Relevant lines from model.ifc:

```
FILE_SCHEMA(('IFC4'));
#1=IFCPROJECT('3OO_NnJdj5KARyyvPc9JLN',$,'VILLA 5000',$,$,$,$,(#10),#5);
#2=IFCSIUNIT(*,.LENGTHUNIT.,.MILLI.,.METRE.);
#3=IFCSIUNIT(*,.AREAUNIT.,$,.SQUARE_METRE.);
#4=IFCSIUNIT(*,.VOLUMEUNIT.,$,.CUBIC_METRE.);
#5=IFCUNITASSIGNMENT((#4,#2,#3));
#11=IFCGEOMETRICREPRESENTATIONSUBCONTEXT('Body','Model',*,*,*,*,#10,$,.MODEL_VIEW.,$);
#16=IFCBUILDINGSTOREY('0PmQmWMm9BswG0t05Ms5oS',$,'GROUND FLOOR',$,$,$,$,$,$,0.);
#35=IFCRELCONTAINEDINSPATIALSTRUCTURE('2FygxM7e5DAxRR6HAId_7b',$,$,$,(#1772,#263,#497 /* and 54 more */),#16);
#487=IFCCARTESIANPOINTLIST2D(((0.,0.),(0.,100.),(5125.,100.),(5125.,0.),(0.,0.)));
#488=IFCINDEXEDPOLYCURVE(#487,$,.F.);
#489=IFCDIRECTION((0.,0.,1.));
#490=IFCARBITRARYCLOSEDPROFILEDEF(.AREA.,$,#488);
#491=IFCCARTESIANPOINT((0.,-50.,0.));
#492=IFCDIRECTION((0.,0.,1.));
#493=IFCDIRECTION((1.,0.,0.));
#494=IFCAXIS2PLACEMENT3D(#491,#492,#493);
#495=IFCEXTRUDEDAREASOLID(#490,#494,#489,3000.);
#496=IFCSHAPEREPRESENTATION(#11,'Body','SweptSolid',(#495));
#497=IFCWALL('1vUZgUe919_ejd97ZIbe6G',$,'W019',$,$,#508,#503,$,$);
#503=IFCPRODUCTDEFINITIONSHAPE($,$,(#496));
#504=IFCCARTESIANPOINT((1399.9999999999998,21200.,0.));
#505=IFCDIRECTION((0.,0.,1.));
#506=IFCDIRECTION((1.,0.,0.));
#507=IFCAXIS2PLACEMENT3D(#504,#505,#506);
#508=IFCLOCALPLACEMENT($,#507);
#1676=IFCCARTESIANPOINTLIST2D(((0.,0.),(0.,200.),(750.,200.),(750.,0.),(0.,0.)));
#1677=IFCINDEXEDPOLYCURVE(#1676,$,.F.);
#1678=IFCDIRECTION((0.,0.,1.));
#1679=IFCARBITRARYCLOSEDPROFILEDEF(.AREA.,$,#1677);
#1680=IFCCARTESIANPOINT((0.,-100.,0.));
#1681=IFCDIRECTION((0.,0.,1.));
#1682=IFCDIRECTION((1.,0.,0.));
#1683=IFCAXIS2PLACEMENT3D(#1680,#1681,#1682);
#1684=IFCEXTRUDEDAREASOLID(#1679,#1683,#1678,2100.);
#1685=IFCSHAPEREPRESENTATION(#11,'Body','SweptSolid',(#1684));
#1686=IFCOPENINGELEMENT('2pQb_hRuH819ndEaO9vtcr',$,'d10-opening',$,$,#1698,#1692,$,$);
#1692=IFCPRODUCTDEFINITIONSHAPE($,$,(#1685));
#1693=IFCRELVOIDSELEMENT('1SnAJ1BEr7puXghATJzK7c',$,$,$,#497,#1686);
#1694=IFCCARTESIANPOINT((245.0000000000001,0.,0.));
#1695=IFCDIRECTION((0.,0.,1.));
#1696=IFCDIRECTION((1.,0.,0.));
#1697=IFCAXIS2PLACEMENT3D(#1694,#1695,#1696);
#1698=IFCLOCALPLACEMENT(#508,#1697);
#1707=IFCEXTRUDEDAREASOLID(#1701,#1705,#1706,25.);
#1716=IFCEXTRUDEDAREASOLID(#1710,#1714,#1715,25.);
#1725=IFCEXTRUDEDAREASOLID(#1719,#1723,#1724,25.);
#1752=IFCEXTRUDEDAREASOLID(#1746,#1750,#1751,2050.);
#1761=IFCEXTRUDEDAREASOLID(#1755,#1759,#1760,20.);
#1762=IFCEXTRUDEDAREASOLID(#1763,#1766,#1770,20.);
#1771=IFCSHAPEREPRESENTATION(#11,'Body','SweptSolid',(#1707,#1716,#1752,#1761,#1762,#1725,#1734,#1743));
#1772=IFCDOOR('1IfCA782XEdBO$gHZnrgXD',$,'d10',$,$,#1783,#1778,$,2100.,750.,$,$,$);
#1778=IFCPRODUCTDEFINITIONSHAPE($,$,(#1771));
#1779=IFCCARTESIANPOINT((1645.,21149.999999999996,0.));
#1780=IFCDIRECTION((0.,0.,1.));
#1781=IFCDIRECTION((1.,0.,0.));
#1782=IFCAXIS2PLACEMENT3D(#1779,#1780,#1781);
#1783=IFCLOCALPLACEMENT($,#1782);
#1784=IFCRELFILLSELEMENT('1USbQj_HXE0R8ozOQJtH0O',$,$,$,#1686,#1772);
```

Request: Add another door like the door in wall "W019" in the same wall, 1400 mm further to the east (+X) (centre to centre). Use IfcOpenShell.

```python
import ifcopenshell
import ifcopenshell.api.feature
import ifcopenshell.api.geometry
import ifcopenshell.api.root
import ifcopenshell.geom
import ifcopenshell.util.element
import ifcopenshell.util.placement
import ifcopenshell.util.shape
import ifcopenshell.util.unit

model = ifcopenshell.open("model.ifc")
unit_scale = ifcopenshell.util.unit.calculate_unit_scale(model)
settings = ifcopenshell.geom.settings()


def volume(element):
    """Net volume in cubic metres, openings subtracted."""
    shape = ifcopenshell.geom.create_shape(settings, element)
    return ifcopenshell.util.shape.get_volume(shape.geometry)


door = model.by_id(1772)
opening = door.FillsVoids[0].RelatingOpeningElement
wall = opening.VoidsElements[0].RelatingBuildingElement
before = volume(wall)
shift = ifcopenshell.util.placement.get_local_placement(wall.ObjectPlacement)[:3, 0] * 1.4 / unit_scale

# copy_class copies the void relationship, type, container and properties, but no geometry.
new_opening = ifcopenshell.api.root.copy_class(model, product=opening)
new_opening.Representation = ifcopenshell.util.element.copy_deep(
    model, opening.Representation, exclude=["IfcGeometricRepresentationContext", "IfcRepresentationMap"]
)
new_door = ifcopenshell.api.root.copy_class(model, product=door)
new_door.Representation = ifcopenshell.util.element.copy_deep(
    model, door.Representation, exclude=["IfcGeometricRepresentationContext", "IfcRepresentationMap"]
)
ifcopenshell.api.feature.add_filling(model, opening=new_opening, element=new_door)

for old, new in ((opening, new_opening), (door, new_door)):
    matrix = ifcopenshell.util.placement.get_local_placement(old.ObjectPlacement)
    matrix[:3, 3] += shift
    ifcopenshell.api.geometry.edit_object_placement(model, product=new, matrix=matrix, is_si=False)

after = volume(wall)

print(f"wall volume {before:.3f} -> {after:.3f} m3")

model.write("model_rev.ifc")
```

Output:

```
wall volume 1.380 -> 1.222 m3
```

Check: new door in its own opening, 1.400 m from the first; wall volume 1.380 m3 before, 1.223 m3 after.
